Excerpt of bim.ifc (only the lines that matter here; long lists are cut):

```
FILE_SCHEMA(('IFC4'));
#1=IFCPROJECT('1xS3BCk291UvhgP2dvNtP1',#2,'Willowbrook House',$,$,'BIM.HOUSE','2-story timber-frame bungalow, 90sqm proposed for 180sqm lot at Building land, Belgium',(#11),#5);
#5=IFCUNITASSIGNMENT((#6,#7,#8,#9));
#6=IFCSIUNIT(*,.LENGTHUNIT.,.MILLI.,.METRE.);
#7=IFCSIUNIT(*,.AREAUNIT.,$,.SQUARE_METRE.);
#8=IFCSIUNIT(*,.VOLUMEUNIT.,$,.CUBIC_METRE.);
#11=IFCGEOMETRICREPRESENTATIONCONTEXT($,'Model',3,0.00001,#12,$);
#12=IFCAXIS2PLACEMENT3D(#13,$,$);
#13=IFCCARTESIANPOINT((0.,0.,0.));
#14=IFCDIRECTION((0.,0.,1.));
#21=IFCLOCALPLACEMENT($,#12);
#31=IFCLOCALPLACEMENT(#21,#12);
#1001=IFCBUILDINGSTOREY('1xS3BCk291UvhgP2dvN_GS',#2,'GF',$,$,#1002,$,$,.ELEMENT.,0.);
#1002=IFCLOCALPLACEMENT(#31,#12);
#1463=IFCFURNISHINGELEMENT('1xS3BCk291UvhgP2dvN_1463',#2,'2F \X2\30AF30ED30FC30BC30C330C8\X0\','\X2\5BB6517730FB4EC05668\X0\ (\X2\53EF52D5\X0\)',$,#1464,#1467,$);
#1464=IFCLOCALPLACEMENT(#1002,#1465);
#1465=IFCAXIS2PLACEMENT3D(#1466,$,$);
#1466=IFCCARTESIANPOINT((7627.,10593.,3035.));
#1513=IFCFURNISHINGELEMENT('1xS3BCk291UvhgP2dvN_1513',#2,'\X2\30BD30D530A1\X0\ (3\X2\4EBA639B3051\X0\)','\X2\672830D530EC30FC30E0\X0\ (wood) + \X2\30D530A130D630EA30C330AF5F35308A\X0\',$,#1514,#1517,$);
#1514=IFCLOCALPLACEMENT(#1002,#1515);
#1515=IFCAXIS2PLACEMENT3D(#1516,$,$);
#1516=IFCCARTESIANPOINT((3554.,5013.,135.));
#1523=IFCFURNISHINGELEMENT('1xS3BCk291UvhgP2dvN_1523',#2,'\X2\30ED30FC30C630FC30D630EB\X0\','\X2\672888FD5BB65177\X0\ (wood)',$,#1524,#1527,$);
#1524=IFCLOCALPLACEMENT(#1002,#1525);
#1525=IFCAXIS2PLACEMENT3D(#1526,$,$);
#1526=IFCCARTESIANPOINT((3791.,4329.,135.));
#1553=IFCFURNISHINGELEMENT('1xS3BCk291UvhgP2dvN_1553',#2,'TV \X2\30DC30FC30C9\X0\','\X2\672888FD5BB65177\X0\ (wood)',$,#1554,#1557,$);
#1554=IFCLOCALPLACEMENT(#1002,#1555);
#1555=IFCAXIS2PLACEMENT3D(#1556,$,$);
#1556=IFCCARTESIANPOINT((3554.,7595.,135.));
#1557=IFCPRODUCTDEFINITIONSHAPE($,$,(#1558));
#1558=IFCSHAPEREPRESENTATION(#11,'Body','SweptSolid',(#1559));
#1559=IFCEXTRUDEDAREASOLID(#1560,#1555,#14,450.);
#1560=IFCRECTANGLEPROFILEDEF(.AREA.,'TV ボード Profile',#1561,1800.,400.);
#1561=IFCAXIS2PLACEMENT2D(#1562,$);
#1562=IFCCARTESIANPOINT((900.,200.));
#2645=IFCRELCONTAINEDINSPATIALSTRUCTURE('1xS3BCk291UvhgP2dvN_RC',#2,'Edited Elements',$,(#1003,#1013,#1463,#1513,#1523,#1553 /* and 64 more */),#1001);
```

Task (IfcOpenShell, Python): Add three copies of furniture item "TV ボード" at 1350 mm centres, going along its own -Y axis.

```python
import ifcopenshell
import ifcopenshell.api.geometry
import ifcopenshell.api.root
import ifcopenshell.util.element
import ifcopenshell.util.placement

model = ifcopenshell.open("bim.ifc")


def reuse_history(source, copy):
    """copy_class also copies each property set's owner history, people and application; keep the originals."""
    for rel in copy.IsDefinedBy:
        if rel.is_a("IfcRelDefinesByProperties") and (history := rel.RelatingPropertyDefinition.OwnerHistory):
            rel.RelatingPropertyDefinition.OwnerHistory = source.OwnerHistory
            ifcopenshell.util.element.remove_deep2(model, history)


source = model.by_guid("1xS3BCk291UvhgP2dvN_1553")
base = ifcopenshell.util.placement.get_local_placement(source.ObjectPlacement)
step = -base[:3, 1] * 1350.0

for i in range(1, 4):
    copy = ifcopenshell.api.root.copy_class(model, product=source)
    copy.Representation = ifcopenshell.util.element.copy_deep(
        model, source.Representation, exclude=["IfcGeometricRepresentationContext", "IfcRepresentationMap"]
    )
    reuse_history(source, copy)
    matrix = base.copy()
    matrix[:3, 3] += i * step
    print("added at", matrix[:3, 3].round(3) + 0.0)
    ifcopenshell.api.geometry.edit_object_placement(model, product=copy, matrix=matrix, is_si=False)

model.write("bim_updated.ifc")
```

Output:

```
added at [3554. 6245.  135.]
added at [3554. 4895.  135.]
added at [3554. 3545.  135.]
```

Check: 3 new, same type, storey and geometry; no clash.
